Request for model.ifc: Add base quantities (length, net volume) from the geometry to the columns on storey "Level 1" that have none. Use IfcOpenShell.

First a look at what the model holds.

```python
import ifcopenshell
import ifcopenshell.util.element
import ifcopenshell.util.unit

model = ifcopenshell.open("model.ifc")
print(model.schema)
for unit_type in ("LENGTHUNIT", "AREAUNIT", "VOLUMEUNIT"):
    print(unit_type, ifcopenshell.util.unit.calculate_unit_scale(model, unit_type))
storey = next(s for s in model.by_type("IfcBuildingStorey") if s.Name == "Level 1")
columns = [e for e in ifcopenshell.util.element.get_decomposition(storey) if e.is_a("IfcColumn")]
for e in sorted(columns, key=lambda e: e.id()):
    print(e.id(), e.is_a(), e.Name, list(ifcopenshell.util.element.get_psets(e, qtos_only=True)), sep=" | ")
```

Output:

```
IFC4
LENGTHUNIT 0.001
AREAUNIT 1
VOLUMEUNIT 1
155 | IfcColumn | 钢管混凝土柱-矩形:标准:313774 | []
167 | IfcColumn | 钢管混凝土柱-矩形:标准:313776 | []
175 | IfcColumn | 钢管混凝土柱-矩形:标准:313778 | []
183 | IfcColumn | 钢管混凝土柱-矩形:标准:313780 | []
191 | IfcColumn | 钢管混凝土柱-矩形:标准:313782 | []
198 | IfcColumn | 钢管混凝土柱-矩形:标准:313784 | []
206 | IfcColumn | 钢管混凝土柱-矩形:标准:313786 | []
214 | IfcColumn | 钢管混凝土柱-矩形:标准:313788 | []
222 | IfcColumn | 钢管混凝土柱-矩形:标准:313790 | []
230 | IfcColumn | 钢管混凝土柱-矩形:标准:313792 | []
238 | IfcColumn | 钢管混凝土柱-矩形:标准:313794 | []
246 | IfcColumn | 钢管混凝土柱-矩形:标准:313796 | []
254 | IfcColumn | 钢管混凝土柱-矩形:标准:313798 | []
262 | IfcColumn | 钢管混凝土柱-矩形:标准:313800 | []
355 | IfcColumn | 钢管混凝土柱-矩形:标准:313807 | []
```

```python
import ifcopenshell
import ifcopenshell.api.pset
import ifcopenshell.geom
import ifcopenshell.util.element
import ifcopenshell.util.shape
import ifcopenshell.util.unit

model = ifcopenshell.open("model.ifc")
unit_scale = ifcopenshell.util.unit.calculate_unit_scale(model)
volume_scale = ifcopenshell.util.unit.calculate_unit_scale(model, "VOLUMEUNIT")
settings = ifcopenshell.geom.settings()

storey = next(s for s in model.by_type("IfcBuildingStorey") if s.Name == "Level 1")
columns = [e for e in ifcopenshell.util.element.get_decomposition(storey) if e.is_a("IfcColumn")]

for e in sorted(columns, key=lambda e: e.id()):
    if ifcopenshell.util.element.get_psets(e, qtos_only=True, should_inherit=False):
        continue
    # Geometry comes back in metres, in the element's own axes.
    shape = ifcopenshell.geom.create_shape(settings, e)
    values = {
        "Length": ifcopenshell.util.shape.get_z(shape.geometry) / unit_scale,
        "NetVolume": ifcopenshell.util.shape.get_volume(shape.geometry) / volume_scale,
    }
    qto = ifcopenshell.api.pset.add_qto(model, product=e, name="Qto_ColumnBaseQuantities")
    ifcopenshell.api.pset.edit_qto(model, qto=qto, properties=values)
    print(e.id(), {k: round(v, 3) for k, v in values.items()})

model.write("model_v2.ifc")
```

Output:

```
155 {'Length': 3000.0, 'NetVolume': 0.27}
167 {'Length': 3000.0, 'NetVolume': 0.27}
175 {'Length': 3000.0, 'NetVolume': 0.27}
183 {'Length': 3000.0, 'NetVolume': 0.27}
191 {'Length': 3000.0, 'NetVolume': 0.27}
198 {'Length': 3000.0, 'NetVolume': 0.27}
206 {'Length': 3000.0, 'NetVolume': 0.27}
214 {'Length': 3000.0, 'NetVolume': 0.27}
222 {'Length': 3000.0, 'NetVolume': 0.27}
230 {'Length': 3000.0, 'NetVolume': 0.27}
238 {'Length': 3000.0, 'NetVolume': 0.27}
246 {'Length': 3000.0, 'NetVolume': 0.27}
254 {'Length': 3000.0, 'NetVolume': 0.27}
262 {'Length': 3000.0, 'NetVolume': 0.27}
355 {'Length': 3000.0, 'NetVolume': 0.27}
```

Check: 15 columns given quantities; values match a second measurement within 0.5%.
